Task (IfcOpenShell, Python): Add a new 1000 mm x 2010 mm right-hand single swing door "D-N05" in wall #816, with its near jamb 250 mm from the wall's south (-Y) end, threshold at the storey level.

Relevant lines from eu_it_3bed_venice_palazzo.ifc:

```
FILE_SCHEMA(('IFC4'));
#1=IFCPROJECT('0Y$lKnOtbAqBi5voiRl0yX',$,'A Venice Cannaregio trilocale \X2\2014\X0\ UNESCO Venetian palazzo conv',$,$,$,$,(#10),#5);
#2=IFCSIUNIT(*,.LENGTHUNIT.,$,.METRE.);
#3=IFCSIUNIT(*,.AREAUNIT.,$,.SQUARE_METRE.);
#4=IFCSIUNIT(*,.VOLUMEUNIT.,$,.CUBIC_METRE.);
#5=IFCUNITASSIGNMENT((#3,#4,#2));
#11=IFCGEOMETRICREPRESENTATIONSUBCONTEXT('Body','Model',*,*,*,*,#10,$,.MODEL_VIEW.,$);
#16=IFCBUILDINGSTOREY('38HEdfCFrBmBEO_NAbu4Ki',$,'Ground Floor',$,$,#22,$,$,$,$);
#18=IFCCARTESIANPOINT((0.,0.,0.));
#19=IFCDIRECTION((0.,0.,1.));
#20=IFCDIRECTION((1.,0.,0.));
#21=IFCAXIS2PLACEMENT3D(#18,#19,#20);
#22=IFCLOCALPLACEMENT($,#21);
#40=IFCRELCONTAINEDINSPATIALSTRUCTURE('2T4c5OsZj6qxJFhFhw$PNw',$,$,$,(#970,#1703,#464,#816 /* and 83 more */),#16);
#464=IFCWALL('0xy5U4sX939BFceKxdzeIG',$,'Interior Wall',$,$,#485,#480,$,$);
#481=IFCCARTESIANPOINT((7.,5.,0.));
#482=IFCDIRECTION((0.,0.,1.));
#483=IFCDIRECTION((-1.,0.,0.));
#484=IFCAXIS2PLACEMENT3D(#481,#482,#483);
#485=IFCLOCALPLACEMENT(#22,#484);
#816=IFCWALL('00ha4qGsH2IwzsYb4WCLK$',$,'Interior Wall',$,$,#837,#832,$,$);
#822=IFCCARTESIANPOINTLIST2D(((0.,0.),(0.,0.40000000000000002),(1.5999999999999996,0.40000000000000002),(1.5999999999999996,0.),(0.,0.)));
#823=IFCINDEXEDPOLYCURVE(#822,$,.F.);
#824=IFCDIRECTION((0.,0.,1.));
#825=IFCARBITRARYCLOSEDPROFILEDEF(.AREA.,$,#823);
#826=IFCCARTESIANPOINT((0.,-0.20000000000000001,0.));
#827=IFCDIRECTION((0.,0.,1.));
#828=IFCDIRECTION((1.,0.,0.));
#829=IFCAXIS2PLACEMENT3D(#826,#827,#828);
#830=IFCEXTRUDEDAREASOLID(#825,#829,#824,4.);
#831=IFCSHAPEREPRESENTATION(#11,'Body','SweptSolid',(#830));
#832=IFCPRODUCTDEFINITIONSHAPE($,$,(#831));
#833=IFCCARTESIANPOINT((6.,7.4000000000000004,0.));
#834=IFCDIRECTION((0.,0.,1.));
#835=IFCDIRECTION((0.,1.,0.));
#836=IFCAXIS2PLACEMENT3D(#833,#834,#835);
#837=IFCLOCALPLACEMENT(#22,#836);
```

```python
import numpy as np
import ifcopenshell
import ifcopenshell.api.feature
import ifcopenshell.api.geometry
import ifcopenshell.api.root
import ifcopenshell.api.spatial
import ifcopenshell.geom
import ifcopenshell.util.element
import ifcopenshell.util.placement
import ifcopenshell.util.representation
import ifcopenshell.util.shape
import ifcopenshell.util.unit

model = ifcopenshell.open("eu_it_3bed_venice_palazzo.ifc")
unit_scale = ifcopenshell.util.unit.calculate_unit_scale(model)
settings = ifcopenshell.geom.settings()


def volume(element):
    """Net volume in cubic metres, openings subtracted."""
    shape = ifcopenshell.geom.create_shape(settings, element)
    return ifcopenshell.util.shape.get_volume(shape.geometry)


wall = model.by_guid("00ha4qGsH2IwzsYb4WCLK$")
storey = ifcopenshell.util.element.get_container(wall, ifc_class="IfcBuildingStorey")
context = ifcopenshell.util.representation.get_context(model, "Model", "Body", "MODEL_VIEW")
before = volume(wall)

width, height, from_end, sill = 1, 2.01, 0.25, 0.0  # metres

# The wall runs along its own X axis, and the end named is its -X end.
wall_shape = ifcopenshell.geom.create_shape(settings, wall)
x, y, z = ifcopenshell.util.shape.get_vertices(wall_shape.geometry).T
start = x.min() + from_end
face, thickness = float(y.min()), float(y.max() - y.min())
wall_matrix = ifcopenshell.util.placement.get_local_placement(wall.ObjectPlacement)
level = ifcopenshell.util.placement.get_local_placement(storey.ObjectPlacement)[2, 3]


def in_wall(x, y):
    """Placement at x, y metres in the wall's axes, at sill height."""
    matrix = wall_matrix.copy()
    matrix[:, 3] = wall_matrix @ np.array([x / unit_scale, y / unit_scale, 0.0, 1.0])
    matrix[2, 3] = level + sill / unit_scale
    return matrix


# Opening: a box that overshoots both wall faces by 50 mm.
opening = ifcopenshell.api.root.create_entity(model, ifc_class="IfcOpeningElement", predefined_type="OPENING")
box = ifcopenshell.api.geometry.add_wall_representation(
    model, context=context, length=width, height=height, thickness=thickness + 0.1
)
ifcopenshell.api.geometry.assign_representation(model, product=opening, representation=box)
ifcopenshell.api.geometry.edit_object_placement(model, product=opening, matrix=in_wall(start, face - 0.05), is_si=False)
ifcopenshell.api.feature.add_feature(model, feature=opening, element=wall)

door = ifcopenshell.api.root.create_entity(model, ifc_class="IfcDoor", name="D-N05", predefined_type="DOOR")
door.OverallWidth, door.OverallHeight = width / unit_scale, height / unit_scale
door.OperationType = "SINGLE_SWING_RIGHT"
body = ifcopenshell.api.geometry.add_door_representation(
    model,
    context=context,
    overall_width=door.OverallWidth,
    overall_height=door.OverallHeight,
    operation_type="SINGLE_SWING_RIGHT",
    lining_properties={"LiningDepth": thickness / unit_scale, "ThresholdDepth": thickness / unit_scale},
)
ifcopenshell.api.geometry.assign_representation(model, product=door, representation=body)
ifcopenshell.api.spatial.assign_container(model, products=[door], relating_structure=storey)
ifcopenshell.api.feature.add_filling(model, opening=opening, element=door)

# The lining spans the wall, so the door starts at the wall face.
ifcopenshell.api.geometry.edit_object_placement(model, product=door, matrix=in_wall(start, face), is_si=False)

after = volume(wall)

print(f"wall volume {before:.3f} -> {after:.3f} m3")

model.write("eu_it_3bed_venice_palazzo-out.ifc")
```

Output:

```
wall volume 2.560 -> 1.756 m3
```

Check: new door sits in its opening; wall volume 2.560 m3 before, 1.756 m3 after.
